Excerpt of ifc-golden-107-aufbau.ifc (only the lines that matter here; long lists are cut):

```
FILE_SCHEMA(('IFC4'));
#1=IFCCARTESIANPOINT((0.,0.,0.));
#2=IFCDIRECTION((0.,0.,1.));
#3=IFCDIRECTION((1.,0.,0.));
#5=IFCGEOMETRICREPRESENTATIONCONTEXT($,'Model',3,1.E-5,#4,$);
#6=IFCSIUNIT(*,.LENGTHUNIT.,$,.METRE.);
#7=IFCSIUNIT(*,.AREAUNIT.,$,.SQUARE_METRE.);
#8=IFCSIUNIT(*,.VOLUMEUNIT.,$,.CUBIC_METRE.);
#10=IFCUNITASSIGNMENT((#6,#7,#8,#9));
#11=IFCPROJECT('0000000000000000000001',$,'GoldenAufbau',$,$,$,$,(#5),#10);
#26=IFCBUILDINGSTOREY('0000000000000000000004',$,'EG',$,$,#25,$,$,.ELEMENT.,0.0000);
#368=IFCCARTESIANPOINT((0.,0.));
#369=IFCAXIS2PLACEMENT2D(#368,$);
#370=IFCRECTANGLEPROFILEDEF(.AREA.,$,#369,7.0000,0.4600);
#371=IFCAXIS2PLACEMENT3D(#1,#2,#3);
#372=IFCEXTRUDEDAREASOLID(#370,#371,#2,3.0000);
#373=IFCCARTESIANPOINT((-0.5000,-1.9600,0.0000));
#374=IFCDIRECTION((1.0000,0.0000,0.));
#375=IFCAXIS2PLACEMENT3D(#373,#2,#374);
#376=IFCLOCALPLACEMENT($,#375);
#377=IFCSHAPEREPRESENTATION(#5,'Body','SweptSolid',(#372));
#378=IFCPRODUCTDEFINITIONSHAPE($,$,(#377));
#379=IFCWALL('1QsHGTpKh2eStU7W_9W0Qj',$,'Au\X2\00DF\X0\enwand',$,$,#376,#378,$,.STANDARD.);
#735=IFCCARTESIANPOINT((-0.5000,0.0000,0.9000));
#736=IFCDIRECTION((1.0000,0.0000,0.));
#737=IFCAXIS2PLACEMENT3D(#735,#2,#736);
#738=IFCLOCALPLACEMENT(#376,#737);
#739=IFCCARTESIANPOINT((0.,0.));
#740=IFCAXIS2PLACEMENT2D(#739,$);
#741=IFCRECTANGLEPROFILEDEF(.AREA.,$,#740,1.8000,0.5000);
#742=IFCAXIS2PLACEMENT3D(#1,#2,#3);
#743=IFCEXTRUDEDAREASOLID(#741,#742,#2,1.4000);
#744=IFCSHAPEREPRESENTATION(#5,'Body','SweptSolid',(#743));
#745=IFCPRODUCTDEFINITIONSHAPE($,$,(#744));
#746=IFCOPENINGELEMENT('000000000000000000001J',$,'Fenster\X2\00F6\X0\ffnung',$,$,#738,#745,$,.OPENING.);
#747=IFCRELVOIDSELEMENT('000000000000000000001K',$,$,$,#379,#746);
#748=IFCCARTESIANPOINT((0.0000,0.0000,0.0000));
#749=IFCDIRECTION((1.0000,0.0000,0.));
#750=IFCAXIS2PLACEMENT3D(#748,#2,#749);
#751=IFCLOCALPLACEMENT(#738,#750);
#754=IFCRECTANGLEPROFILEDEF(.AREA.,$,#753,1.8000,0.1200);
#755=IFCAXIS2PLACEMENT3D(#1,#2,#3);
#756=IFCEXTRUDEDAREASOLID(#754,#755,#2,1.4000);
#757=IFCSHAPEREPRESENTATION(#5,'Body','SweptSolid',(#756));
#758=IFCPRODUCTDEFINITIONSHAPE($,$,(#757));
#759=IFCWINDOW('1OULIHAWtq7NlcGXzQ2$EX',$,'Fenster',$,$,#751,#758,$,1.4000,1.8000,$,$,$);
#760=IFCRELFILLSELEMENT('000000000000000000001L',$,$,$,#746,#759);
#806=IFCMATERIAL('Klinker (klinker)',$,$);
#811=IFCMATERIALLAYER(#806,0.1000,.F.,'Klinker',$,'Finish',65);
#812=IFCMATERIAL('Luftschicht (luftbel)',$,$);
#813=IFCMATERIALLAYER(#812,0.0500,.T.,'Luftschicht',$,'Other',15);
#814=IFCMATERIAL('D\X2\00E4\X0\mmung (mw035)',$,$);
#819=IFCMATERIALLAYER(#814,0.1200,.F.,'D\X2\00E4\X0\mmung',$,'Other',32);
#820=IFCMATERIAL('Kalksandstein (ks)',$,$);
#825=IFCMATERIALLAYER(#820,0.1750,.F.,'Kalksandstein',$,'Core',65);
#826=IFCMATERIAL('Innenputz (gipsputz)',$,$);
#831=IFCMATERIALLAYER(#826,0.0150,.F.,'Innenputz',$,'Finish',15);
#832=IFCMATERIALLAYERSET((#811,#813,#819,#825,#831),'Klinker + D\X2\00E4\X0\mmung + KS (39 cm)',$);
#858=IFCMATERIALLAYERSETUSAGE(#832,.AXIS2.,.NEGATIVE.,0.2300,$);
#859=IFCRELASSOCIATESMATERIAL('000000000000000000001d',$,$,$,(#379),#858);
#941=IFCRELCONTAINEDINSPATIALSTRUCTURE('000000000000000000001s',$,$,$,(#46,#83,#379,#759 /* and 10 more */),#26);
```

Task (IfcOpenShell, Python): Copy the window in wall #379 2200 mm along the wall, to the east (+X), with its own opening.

```python
import ifcopenshell
import ifcopenshell.api.feature
import ifcopenshell.api.geometry
import ifcopenshell.api.root
import ifcopenshell.geom
import ifcopenshell.util.element
import ifcopenshell.util.placement
import ifcopenshell.util.shape
import ifcopenshell.util.unit

model = ifcopenshell.open("ifc-golden-107-aufbau.ifc")
unit_scale = ifcopenshell.util.unit.calculate_unit_scale(model)
settings = ifcopenshell.geom.settings()


def volume(element):
    """Net volume in cubic metres, openings subtracted."""
    shape = ifcopenshell.geom.create_shape(settings, element)
    return ifcopenshell.util.shape.get_volume(shape.geometry)


window = model.by_guid("1OULIHAWtq7NlcGXzQ2$EX")
opening = window.FillsVoids[0].RelatingOpeningElement
wall = opening.VoidsElements[0].RelatingBuildingElement
before = volume(wall)
shift = ifcopenshell.util.placement.get_local_placement(wall.ObjectPlacement)[:3, 0] * 2.2 / unit_scale

# copy_class copies the void relationship, type, container and properties, but no geometry.
new_opening = ifcopenshell.api.root.copy_class(model, product=opening)
new_opening.Representation = ifcopenshell.util.element.copy_deep(
    model, opening.Representation, exclude=["IfcGeometricRepresentationContext", "IfcRepresentationMap"]
)
new_window = ifcopenshell.api.root.copy_class(model, product=window)
new_window.Representation = ifcopenshell.util.element.copy_deep(
    model, window.Representation, exclude=["IfcGeometricRepresentationContext", "IfcRepresentationMap"]
)
ifcopenshell.api.feature.add_filling(model, opening=new_opening, element=new_window)

for old, new in ((opening, new_opening), (window, new_window)):
    matrix = ifcopenshell.util.placement.get_local_placement(old.ObjectPlacement)
    matrix[:3, 3] += shift
    ifcopenshell.api.geometry.edit_object_placement(model, product=new, matrix=matrix, is_si=False)

after = volume(wall)

print(f"wall volume {before:.3f} -> {after:.3f} m3")

model.write("ifc-golden-107-aufbau_edited.ifc")
```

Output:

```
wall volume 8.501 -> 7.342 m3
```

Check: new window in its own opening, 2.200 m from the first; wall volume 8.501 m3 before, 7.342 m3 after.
